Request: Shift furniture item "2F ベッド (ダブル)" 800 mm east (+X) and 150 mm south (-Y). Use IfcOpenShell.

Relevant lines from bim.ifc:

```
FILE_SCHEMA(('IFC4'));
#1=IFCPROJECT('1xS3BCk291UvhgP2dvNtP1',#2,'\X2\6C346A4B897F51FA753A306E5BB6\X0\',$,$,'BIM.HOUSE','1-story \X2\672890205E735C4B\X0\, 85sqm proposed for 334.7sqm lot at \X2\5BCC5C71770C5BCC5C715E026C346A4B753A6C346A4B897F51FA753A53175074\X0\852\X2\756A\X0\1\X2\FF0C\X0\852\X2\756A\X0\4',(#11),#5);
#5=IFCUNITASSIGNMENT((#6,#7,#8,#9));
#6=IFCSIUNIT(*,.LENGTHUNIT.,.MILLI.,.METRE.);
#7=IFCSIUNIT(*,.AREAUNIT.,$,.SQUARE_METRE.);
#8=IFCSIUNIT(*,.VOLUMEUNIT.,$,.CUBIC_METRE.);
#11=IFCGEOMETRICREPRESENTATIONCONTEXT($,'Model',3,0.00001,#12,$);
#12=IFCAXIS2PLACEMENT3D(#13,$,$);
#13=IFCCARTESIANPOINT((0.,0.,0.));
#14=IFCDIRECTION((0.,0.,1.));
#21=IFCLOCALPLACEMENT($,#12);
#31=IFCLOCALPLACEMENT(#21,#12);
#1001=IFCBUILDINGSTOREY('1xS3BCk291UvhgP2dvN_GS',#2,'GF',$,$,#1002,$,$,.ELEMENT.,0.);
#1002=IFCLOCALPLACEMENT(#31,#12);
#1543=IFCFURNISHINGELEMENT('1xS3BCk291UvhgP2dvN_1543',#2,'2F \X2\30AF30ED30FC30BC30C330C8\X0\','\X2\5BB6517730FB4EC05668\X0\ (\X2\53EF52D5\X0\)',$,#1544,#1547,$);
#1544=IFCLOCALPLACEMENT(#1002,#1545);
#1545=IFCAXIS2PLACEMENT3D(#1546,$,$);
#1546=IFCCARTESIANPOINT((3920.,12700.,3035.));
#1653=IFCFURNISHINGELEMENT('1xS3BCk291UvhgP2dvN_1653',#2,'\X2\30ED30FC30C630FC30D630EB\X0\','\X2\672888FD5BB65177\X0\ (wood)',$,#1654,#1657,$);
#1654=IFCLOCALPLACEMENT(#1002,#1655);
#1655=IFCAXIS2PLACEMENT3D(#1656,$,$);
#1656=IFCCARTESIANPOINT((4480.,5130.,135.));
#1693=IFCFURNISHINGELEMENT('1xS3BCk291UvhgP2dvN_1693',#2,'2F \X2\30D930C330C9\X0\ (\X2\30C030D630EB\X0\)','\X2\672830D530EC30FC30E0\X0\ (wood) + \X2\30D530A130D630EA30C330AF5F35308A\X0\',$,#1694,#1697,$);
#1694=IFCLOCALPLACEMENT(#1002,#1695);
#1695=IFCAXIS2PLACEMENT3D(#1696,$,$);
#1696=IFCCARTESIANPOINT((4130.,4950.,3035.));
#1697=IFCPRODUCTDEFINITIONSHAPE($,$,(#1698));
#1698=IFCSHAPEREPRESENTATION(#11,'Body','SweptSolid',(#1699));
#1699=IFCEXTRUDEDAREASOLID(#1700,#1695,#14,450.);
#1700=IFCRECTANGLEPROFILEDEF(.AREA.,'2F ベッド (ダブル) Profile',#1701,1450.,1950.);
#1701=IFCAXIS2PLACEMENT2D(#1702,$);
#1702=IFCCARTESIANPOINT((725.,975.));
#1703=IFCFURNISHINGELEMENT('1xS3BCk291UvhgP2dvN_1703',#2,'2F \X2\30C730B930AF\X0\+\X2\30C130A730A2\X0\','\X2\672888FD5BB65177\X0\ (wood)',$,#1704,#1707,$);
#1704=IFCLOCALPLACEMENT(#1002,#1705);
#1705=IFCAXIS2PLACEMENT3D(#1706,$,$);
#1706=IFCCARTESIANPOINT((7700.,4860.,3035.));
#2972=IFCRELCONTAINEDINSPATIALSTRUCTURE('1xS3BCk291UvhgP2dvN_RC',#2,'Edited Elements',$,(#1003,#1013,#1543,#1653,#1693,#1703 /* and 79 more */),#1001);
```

```python
import ifcopenshell
import ifcopenshell.api.geometry
import ifcopenshell.util.placement

model = ifcopenshell.open("bim.ifc")

item = model.by_id(1693)
matrix = ifcopenshell.util.placement.get_local_placement(item.ObjectPlacement)
matrix[0, 3] += 800.0
matrix[1, 3] -= 150.0
ifcopenshell.api.geometry.edit_object_placement(model, product=item, matrix=matrix, is_si=False)

print(ifcopenshell.util.placement.get_local_placement(item.ObjectPlacement).round(3) + 0.0)

model.write("bim_rev.ifc")
```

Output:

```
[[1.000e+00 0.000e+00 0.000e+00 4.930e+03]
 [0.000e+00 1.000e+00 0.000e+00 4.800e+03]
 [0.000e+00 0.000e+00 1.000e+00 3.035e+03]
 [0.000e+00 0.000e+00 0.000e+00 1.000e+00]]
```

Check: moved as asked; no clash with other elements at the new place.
